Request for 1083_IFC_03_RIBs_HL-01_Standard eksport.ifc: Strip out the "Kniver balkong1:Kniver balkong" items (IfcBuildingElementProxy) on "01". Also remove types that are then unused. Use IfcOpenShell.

First a look at what the model holds.

```python
import ifcopenshell
import ifcopenshell.util.element

model = ifcopenshell.open("1083_IFC_03_RIBs_HL-01_Standard eksport.ifc")
print(model.schema)
storey = next(s for s in model.by_type("IfcBuildingStorey") if s.Name == "01")
proxies = [e for e in ifcopenshell.util.element.get_decomposition(storey) if e.is_a("IfcBuildingElementProxy")]
seen = {}
for e in proxies:
    element_type = ifcopenshell.util.element.get_type(e)
    name = element_type.Name if element_type not in (None, e) else None
    seen[name] = seen.get(name, 0) + 1
for name, count in sorted(seen.items(), key=str):
    print(count, "x", name)
```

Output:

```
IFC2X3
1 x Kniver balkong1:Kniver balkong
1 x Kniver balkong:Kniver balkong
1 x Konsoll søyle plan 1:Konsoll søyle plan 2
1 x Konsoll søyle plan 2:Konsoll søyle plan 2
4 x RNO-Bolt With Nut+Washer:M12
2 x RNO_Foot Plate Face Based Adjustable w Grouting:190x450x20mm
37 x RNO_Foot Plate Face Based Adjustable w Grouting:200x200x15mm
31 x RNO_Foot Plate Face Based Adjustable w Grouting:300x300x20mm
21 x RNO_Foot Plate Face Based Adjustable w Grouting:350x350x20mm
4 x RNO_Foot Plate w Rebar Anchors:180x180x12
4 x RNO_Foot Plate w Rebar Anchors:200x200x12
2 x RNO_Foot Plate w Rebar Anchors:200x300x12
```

```python
import ifcopenshell
import ifcopenshell.api.root
import ifcopenshell.util.element

model = ifcopenshell.open("1083_IFC_03_RIBs_HL-01_Standard eksport.ifc")

storey = next(s for s in model.by_type("IfcBuildingStorey") if s.Name == "01")
proxies = [e for e in ifcopenshell.util.element.get_decomposition(storey) if e.is_a("IfcBuildingElementProxy")]
targets = [e for e in proxies if (t := ifcopenshell.util.element.get_type(e)) not in (None, e) and t.Name == "Kniver balkong1:Kniver balkong"]
types = {ifcopenshell.util.element.get_type(e) for e in targets} - {None, *targets}

for e in targets:
    ifcopenshell.api.root.remove_product(model, product=e)
print(len(targets), "removed")

unused = [t for t in types if not ifcopenshell.util.element.get_types(t)]
for t in unused:
    ifcopenshell.api.root.remove_product(model, product=t)
print(len(unused), "unused types removed")

model.write("1083_IFC_03_RIBs_HL-01_Standard eksport_rev.ifc")
```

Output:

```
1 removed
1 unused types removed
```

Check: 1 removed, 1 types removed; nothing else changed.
